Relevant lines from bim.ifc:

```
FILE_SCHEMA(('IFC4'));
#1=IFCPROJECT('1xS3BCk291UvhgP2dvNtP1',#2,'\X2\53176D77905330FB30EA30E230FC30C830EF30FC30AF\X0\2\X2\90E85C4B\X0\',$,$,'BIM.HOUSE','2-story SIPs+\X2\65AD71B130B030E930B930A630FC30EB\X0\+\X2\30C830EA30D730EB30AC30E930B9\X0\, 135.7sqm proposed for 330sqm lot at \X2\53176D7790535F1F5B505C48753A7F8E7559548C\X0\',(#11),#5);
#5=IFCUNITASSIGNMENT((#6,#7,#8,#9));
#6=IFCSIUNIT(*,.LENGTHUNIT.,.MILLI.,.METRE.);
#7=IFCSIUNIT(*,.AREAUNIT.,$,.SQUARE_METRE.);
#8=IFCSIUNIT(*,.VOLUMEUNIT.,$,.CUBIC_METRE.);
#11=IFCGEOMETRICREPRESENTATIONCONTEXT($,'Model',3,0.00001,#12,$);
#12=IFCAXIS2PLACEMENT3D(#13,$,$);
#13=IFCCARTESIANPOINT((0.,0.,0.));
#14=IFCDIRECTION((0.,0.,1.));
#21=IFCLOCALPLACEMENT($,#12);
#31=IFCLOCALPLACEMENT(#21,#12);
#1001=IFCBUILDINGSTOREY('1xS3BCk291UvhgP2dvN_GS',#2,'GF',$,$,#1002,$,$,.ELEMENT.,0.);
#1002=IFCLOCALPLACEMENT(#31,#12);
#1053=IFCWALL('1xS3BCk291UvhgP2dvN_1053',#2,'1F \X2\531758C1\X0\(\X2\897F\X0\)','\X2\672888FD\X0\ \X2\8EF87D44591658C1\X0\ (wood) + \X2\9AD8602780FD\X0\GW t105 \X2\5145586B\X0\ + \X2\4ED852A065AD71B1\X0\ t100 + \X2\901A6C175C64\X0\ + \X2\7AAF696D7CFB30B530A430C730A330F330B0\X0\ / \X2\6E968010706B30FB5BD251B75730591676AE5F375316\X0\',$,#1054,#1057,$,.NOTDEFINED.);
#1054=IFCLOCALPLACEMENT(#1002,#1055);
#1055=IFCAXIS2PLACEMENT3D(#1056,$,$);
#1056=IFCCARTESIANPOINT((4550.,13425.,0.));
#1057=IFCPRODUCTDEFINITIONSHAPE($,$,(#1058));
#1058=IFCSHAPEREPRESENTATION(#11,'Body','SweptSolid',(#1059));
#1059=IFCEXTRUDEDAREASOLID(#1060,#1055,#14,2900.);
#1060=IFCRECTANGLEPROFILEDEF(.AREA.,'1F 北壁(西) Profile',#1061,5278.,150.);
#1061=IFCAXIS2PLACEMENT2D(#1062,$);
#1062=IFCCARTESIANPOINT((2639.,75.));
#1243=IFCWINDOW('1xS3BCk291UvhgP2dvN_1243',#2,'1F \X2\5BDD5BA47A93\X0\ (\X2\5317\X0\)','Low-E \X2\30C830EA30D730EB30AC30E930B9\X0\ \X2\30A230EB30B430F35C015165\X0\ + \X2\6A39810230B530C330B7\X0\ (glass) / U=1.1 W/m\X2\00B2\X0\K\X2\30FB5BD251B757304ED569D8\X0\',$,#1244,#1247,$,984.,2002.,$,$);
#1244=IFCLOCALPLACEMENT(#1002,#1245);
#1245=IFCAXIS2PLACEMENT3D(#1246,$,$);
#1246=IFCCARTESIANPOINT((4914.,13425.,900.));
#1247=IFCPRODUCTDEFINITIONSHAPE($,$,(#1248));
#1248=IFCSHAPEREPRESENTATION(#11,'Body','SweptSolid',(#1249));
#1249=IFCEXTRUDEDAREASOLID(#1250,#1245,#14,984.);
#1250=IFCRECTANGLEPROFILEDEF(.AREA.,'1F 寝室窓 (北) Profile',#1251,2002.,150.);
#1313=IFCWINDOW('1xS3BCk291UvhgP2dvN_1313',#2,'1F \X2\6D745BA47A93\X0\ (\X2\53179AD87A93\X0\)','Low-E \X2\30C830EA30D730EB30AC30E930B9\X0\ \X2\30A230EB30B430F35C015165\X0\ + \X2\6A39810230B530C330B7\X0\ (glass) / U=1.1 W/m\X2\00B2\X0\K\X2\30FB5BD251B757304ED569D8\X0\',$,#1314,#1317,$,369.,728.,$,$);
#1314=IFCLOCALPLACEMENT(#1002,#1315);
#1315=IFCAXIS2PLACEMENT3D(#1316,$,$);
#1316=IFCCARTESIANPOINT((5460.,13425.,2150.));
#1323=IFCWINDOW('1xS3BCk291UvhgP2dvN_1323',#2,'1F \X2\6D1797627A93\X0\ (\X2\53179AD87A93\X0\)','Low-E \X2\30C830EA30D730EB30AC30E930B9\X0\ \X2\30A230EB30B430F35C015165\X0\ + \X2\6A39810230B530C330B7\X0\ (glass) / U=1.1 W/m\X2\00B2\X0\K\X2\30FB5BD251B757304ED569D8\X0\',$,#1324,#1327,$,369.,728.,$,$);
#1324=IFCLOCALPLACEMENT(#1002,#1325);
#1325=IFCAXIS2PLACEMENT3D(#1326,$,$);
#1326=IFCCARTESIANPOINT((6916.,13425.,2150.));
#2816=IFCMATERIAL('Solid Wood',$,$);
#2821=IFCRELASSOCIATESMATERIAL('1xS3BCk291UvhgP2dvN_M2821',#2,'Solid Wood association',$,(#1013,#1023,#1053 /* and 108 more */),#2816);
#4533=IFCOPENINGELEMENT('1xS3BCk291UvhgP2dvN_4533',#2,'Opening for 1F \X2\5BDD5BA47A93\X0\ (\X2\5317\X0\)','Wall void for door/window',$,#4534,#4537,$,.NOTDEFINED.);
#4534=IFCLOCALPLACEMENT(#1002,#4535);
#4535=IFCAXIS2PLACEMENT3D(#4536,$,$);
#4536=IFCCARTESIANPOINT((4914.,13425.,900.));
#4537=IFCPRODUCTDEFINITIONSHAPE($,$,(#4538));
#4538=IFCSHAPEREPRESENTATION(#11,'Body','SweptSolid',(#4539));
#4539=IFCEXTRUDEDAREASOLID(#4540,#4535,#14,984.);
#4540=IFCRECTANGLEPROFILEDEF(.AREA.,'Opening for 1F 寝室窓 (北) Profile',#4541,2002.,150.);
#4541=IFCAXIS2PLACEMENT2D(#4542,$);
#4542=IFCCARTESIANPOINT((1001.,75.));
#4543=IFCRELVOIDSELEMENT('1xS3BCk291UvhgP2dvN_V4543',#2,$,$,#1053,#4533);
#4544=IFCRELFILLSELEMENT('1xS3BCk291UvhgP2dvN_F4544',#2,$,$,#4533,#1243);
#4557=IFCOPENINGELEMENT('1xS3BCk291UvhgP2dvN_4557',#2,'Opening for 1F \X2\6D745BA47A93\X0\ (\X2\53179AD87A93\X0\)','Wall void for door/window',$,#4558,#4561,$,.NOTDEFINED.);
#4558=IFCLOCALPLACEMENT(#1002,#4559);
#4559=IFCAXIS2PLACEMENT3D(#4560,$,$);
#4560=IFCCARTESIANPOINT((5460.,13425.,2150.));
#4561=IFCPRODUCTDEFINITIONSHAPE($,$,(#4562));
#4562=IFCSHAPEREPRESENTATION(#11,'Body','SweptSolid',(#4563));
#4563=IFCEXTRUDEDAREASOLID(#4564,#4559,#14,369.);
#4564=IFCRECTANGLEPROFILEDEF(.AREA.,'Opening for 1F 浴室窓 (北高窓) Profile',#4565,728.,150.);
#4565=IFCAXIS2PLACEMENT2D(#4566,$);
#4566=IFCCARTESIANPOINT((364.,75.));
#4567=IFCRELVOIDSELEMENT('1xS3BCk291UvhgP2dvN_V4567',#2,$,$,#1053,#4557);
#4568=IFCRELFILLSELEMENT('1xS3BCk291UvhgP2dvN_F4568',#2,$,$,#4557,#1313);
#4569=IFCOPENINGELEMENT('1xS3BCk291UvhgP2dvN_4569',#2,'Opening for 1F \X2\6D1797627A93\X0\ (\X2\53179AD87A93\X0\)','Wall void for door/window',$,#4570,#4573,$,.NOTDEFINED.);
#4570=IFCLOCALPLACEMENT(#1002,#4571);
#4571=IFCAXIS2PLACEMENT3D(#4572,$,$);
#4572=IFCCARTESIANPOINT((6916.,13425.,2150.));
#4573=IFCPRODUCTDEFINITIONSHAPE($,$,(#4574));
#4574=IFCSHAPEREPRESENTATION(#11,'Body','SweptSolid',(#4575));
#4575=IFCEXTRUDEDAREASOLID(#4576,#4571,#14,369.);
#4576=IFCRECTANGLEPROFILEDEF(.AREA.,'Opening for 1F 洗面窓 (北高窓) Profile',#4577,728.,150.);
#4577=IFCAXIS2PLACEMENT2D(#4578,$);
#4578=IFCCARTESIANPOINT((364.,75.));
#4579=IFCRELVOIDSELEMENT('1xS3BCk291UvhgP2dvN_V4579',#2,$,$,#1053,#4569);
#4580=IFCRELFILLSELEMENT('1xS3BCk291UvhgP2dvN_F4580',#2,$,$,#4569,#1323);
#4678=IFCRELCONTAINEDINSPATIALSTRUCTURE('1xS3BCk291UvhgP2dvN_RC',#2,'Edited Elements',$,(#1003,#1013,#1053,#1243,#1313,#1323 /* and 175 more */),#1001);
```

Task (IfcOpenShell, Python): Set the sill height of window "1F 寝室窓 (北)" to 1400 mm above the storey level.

```python
import numpy as np
import ifcopenshell
import ifcopenshell.api.geometry
import ifcopenshell.geom
import ifcopenshell.util.element
import ifcopenshell.util.placement
import ifcopenshell.util.shape
import ifcopenshell.util.unit

model = ifcopenshell.open("bim.ifc")
unit_scale = ifcopenshell.util.unit.calculate_unit_scale(model)

window = model.by_id(1243)
opening = window.FillsVoids[0].RelatingOpeningElement
storey = ifcopenshell.util.element.get_container(window, ifc_class="IfcBuildingStorey")
level = ifcopenshell.util.placement.get_local_placement(storey.ObjectPlacement)[2, 3]

# The opening's origin need not be at the sill, so measure its lowest point.
shape = ifcopenshell.geom.create_shape(ifcopenshell.geom.settings(), opening)
bottom = ifcopenshell.util.shape.get_shape_bottom_elevation(shape, shape.geometry) / unit_scale
dz = level + 1.4 / unit_scale - bottom

shift = np.array([0.0, 0.0, dz])
# The window is not placed relative to its opening, so move both.
for product in (opening, window):
    matrix = ifcopenshell.util.placement.get_local_placement(product.ObjectPlacement)
    matrix[:3, 3] += shift
    ifcopenshell.api.geometry.edit_object_placement(model, product=product, matrix=matrix, is_si=False)

print(f"moved by {dz * unit_scale:+.3f} m")

model.write("bim_edited.ifc")
```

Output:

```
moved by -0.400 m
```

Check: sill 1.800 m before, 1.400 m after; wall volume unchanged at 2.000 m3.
